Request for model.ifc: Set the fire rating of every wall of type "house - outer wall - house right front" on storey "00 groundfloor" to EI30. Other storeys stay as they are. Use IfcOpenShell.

First a look at what the model holds.

```python
import ifcopenshell
import ifcopenshell.util.element

model = ifcopenshell.open("model.ifc")
print(model.schema)
storey = next(s for s in model.by_type("IfcBuildingStorey") if s.Name == "00 groundfloor")
walls = [e for e in ifcopenshell.util.element.get_decomposition(storey) if e.is_a("IfcWall")]
seen = {}
for e in walls:
    element_type = ifcopenshell.util.element.get_type(e)
    key = (element_type.Name if element_type != e and element_type else None, ifcopenshell.util.element.get_pset(e, "Pset_WallCommon", "FireRating"))
    seen[key] = seen.get(key, 0) + 1
for (name, value), count in sorted(seen.items(), key=str):
    print(count, "x", name, "|", value)
```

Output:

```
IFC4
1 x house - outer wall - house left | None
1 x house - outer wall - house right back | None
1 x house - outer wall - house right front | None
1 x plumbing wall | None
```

```python
import ifcopenshell
import ifcopenshell.api.pset
import ifcopenshell.util.element

model = ifcopenshell.open("model.ifc")

storey = next(s for s in model.by_type("IfcBuildingStorey") if s.Name == "00 groundfloor")
walls = [e for e in ifcopenshell.util.element.get_decomposition(storey) if e.is_a("IfcWall")]

count = 0
for e in walls:
    element_type = ifcopenshell.util.element.get_type(e)
    if element_type in (None, e) or element_type.Name != "house - outer wall - house right front":
        continue
    # add_pset returns the element's existing set when there is one.
    pset = ifcopenshell.api.pset.add_pset(model, product=e, name="Pset_WallCommon")
    ifcopenshell.api.pset.edit_pset(model, pset=pset, properties={"FireRating": "EI30"})
    count += 1

print(count, "walls updated")

model.write("model_v2.ifc")
```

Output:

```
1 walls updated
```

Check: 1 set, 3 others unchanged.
